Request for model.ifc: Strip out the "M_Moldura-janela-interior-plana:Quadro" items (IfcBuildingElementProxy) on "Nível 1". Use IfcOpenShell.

First a look at what the model holds.

```python
import ifcopenshell
import ifcopenshell.util.element

model = ifcopenshell.open("model.ifc")
print(model.schema)
storey = next(s for s in model.by_type("IfcBuildingStorey") if s.Name == "Nível 1")
proxies = [e for e in ifcopenshell.util.element.get_decomposition(storey) if e.is_a("IfcBuildingElementProxy")]
seen = {}
for e in proxies:
    element_type = ifcopenshell.util.element.get_type(e)
    name = element_type.Name if element_type not in (None, e) else None
    seen[name] = seen.get(name, 0) + 1
for name, count in sorted(seen.items(), key=str):
    print(count, "x", name)
```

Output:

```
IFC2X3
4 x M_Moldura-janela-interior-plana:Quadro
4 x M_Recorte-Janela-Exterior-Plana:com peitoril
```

```python
import ifcopenshell
import ifcopenshell.api.root
import ifcopenshell.util.element

model = ifcopenshell.open("model.ifc")

storey = next(s for s in model.by_type("IfcBuildingStorey") if s.Name == "Nível 1")
proxies = [e for e in ifcopenshell.util.element.get_decomposition(storey) if e.is_a("IfcBuildingElementProxy")]
targets = [e for e in proxies if (t := ifcopenshell.util.element.get_type(e)) not in (None, e) and t.Name == "M_Moldura-janela-interior-plana:Quadro"]

for e in targets:
    ifcopenshell.api.root.remove_product(model, product=e)
print(len(targets), "removed")

model.write("model_rev.ifc")
```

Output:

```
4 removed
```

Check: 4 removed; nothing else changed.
